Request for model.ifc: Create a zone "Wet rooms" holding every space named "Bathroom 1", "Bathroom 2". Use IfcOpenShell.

First a look at what the model holds.

```python
import ifcopenshell

model = ifcopenshell.open("model.ifc")
print(model.schema)
seen = {}
for space in model.by_type("IfcSpace"):
    seen[space.LongName] = seen.get(space.LongName, 0) + 1
for name, count in sorted(seen.items(), key=str):
    print(count, "x", name)
print("zones:", [z.Name for z in model.by_type("IfcZone")][:20])
```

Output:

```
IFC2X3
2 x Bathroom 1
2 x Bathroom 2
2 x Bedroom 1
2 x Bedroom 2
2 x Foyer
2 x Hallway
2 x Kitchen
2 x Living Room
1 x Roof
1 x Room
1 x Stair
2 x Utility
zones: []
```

```python
import ifcopenshell
import ifcopenshell.api.group
import ifcopenshell.api.root

model = ifcopenshell.open("model.ifc")

names = {"Bathroom 1", "Bathroom 2"}
spaces = [s for s in model.by_type("IfcSpace") if s.LongName in names]

zone = ifcopenshell.api.root.create_entity(model, ifc_class="IfcZone", name="Wet rooms")
ifcopenshell.api.group.assign_group(model, products=spaces, group=zone)
print(len(spaces), "spaces in", zone.Name)

model.write("model_updated.ifc")
```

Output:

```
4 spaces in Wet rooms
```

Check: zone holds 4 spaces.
